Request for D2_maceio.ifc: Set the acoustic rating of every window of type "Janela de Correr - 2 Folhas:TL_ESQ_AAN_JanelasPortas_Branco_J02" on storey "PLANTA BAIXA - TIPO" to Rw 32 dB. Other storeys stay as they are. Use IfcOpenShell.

First a look at what the model holds.

```python
import ifcopenshell
import ifcopenshell.util.element

model = ifcopenshell.open("D2_maceio.ifc")
print(model.schema)
storey = next(s for s in model.by_type("IfcBuildingStorey") if s.Name == "PLANTA BAIXA - TIPO")
windows = [e for e in ifcopenshell.util.element.get_decomposition(storey) if e.is_a("IfcWindow")]
seen = {}
for e in windows:
    element_type = ifcopenshell.util.element.get_type(e)
    key = (element_type.Name if element_type != e and element_type else None, ifcopenshell.util.element.get_pset(e, "Pset_WindowCommon", "AcousticRating"))
    seen[key] = seen.get(key, 0) + 1
for (name, value), count in sorted(seen.items(), key=str):
    print(count, "x", name, "|", value)
```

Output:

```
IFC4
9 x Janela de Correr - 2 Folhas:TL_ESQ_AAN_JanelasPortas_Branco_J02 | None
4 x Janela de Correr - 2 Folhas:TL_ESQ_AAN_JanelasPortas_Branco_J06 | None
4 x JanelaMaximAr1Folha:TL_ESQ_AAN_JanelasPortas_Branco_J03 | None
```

```python
import ifcopenshell
import ifcopenshell.api.pset
import ifcopenshell.util.element

model = ifcopenshell.open("D2_maceio.ifc")

storey = next(s for s in model.by_type("IfcBuildingStorey") if s.Name == "PLANTA BAIXA - TIPO")
windows = [e for e in ifcopenshell.util.element.get_decomposition(storey) if e.is_a("IfcWindow")]

count = 0
for e in windows:
    element_type = ifcopenshell.util.element.get_type(e)
    if element_type in (None, e) or element_type.Name != "Janela de Correr - 2 Folhas:TL_ESQ_AAN_JanelasPortas_Branco_J02":
        continue
    # add_pset returns the element's existing set when there is one.
    pset = ifcopenshell.api.pset.add_pset(model, product=e, name="Pset_WindowCommon")
    ifcopenshell.api.pset.edit_pset(model, pset=pset, properties={"AcousticRating": "Rw 32 dB"})
    count += 1

print(count, "windows updated")

model.write("D2_maceio_updated.ifc")
```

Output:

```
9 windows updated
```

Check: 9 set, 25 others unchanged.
